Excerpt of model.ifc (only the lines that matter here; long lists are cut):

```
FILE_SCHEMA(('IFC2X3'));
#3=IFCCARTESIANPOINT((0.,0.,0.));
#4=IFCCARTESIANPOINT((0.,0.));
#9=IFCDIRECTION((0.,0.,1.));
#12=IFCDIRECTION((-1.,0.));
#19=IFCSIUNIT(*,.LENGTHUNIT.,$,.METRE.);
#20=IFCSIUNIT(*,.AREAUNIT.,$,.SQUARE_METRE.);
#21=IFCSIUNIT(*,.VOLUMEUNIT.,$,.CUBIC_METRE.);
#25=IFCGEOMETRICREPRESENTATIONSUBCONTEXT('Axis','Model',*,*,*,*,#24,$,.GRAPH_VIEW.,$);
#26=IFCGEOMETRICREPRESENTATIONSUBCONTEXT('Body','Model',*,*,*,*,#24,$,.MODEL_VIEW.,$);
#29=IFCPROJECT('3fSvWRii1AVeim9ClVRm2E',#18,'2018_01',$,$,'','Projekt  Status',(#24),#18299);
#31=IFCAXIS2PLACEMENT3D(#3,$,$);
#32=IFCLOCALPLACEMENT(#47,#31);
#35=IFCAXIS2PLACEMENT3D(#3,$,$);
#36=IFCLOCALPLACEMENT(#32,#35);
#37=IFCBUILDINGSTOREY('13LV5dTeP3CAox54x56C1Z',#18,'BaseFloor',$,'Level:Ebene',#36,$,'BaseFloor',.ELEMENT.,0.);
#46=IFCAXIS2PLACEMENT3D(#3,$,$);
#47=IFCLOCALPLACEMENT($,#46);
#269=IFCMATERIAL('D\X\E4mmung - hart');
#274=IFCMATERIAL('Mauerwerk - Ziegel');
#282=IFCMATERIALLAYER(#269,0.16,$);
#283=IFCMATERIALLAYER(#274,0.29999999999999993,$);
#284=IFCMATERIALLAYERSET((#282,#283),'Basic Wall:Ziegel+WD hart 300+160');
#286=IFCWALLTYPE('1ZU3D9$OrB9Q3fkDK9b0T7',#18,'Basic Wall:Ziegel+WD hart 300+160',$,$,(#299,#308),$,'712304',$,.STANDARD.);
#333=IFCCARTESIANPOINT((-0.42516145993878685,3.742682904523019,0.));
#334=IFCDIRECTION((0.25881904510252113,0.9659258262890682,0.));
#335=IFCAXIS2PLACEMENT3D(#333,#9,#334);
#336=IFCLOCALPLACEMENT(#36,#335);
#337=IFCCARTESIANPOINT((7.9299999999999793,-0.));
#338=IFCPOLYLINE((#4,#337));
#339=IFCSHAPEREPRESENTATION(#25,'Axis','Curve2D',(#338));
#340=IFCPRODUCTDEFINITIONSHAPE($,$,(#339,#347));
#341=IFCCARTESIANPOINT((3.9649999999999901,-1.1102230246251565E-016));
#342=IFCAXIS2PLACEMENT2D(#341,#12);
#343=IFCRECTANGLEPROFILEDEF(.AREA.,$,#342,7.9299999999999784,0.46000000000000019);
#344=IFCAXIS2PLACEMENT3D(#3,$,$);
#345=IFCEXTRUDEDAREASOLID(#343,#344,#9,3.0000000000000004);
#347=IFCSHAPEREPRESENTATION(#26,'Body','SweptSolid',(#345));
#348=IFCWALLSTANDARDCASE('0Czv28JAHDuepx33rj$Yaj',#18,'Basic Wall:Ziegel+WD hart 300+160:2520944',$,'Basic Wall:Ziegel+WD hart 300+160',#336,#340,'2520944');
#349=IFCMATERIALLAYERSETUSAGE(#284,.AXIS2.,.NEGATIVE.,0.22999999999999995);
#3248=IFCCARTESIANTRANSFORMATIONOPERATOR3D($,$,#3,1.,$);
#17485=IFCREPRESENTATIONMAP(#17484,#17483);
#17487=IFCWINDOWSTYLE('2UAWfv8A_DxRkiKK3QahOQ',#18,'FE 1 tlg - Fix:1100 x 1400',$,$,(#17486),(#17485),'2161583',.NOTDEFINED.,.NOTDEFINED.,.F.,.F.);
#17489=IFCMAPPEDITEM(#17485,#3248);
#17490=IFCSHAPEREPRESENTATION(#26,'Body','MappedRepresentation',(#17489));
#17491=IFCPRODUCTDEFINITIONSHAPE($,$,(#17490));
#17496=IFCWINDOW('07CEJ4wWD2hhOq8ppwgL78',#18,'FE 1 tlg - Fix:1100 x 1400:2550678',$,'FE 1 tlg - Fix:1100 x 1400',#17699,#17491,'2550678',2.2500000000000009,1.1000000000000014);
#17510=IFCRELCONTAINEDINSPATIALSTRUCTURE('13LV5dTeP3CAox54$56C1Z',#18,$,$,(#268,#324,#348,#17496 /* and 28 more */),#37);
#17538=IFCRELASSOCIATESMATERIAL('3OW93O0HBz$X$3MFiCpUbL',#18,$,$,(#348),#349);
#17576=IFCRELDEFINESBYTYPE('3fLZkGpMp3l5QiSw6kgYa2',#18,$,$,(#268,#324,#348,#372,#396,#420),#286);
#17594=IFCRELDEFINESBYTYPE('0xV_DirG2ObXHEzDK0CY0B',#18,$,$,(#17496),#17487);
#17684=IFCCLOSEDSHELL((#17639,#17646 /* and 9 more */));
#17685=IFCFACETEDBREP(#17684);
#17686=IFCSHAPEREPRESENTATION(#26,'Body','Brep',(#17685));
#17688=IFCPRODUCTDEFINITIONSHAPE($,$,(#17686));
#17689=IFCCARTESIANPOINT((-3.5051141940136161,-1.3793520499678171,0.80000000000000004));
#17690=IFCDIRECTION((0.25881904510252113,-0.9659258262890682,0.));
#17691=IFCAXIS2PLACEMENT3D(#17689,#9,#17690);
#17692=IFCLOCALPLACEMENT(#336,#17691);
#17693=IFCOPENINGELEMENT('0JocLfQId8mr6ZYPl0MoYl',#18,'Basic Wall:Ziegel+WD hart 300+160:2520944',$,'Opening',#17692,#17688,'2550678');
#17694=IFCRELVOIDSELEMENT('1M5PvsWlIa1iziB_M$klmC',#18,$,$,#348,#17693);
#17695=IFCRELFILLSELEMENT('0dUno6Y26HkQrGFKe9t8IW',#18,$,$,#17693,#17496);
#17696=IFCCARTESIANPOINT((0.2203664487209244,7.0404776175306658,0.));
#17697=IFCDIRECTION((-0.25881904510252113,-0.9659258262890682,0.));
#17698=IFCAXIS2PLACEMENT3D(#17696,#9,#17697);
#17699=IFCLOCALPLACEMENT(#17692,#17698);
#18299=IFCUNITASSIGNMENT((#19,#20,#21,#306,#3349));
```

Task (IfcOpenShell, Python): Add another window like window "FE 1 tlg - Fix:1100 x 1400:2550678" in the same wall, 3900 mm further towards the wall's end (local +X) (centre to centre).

```python
import ifcopenshell
import ifcopenshell.api.feature
import ifcopenshell.api.geometry
import ifcopenshell.api.root
import ifcopenshell.geom
import ifcopenshell.util.element
import ifcopenshell.util.placement
import ifcopenshell.util.shape
import ifcopenshell.util.unit

model = ifcopenshell.open("model.ifc")
unit_scale = ifcopenshell.util.unit.calculate_unit_scale(model)
settings = ifcopenshell.geom.settings()


def volume(element):
    """Net volume in cubic metres, openings subtracted."""
    shape = ifcopenshell.geom.create_shape(settings, element)
    return ifcopenshell.util.shape.get_volume(shape.geometry)


def reuse_history(source, copy):
    """copy_class also copies each property set's owner history, people and application; keep the originals."""
    for rel in copy.IsDefinedBy:
        if rel.is_a("IfcRelDefinesByProperties") and (history := rel.RelatingPropertyDefinition.OwnerHistory):
            rel.RelatingPropertyDefinition.OwnerHistory = source.OwnerHistory
            ifcopenshell.util.element.remove_deep2(model, history)


window = model.by_guid("07CEJ4wWD2hhOq8ppwgL78")
opening = window.FillsVoids[0].RelatingOpeningElement
wall = opening.VoidsElements[0].RelatingBuildingElement
before = volume(wall)
shift = ifcopenshell.util.placement.get_local_placement(wall.ObjectPlacement)[:3, 0] * 3.9 / unit_scale

# copy_class copies the void relationship, type, container and properties, but no geometry.
new_opening = ifcopenshell.api.root.copy_class(model, product=opening)
new_opening.Representation = ifcopenshell.util.element.copy_deep(
    model, opening.Representation, exclude=["IfcGeometricRepresentationContext", "IfcRepresentationMap"]
)
new_opening.Name = "Basic Wall:Ziegel+WD hart 300+160"
new_opening.Tag = None
new_window = ifcopenshell.api.root.copy_class(model, product=window)
new_window.Representation = ifcopenshell.util.element.copy_deep(
    model, window.Representation, exclude=["IfcGeometricRepresentationContext", "IfcRepresentationMap"]
)
new_window.Name = "FE 1 tlg - Fix:1100 x 1400"
new_window.Tag = None
reuse_history(window, new_window)
fills = ifcopenshell.api.feature.add_filling(model, opening=new_opening, element=new_window)
fills.OwnerHistory = new_window.OwnerHistory  # required in IFC2X3

for old, new in ((opening, new_opening), (window, new_window)):
    matrix = ifcopenshell.util.placement.get_local_placement(old.ObjectPlacement)
    matrix[:3, 3] += shift
    ifcopenshell.api.geometry.edit_object_placement(model, product=new, matrix=matrix, is_si=False)

after = volume(wall)

print(f"wall volume {before:.3f} -> {after:.3f} m3")

model.write("model_updated.ifc")
```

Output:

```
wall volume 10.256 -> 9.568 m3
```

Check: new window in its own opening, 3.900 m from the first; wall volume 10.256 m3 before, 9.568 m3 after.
